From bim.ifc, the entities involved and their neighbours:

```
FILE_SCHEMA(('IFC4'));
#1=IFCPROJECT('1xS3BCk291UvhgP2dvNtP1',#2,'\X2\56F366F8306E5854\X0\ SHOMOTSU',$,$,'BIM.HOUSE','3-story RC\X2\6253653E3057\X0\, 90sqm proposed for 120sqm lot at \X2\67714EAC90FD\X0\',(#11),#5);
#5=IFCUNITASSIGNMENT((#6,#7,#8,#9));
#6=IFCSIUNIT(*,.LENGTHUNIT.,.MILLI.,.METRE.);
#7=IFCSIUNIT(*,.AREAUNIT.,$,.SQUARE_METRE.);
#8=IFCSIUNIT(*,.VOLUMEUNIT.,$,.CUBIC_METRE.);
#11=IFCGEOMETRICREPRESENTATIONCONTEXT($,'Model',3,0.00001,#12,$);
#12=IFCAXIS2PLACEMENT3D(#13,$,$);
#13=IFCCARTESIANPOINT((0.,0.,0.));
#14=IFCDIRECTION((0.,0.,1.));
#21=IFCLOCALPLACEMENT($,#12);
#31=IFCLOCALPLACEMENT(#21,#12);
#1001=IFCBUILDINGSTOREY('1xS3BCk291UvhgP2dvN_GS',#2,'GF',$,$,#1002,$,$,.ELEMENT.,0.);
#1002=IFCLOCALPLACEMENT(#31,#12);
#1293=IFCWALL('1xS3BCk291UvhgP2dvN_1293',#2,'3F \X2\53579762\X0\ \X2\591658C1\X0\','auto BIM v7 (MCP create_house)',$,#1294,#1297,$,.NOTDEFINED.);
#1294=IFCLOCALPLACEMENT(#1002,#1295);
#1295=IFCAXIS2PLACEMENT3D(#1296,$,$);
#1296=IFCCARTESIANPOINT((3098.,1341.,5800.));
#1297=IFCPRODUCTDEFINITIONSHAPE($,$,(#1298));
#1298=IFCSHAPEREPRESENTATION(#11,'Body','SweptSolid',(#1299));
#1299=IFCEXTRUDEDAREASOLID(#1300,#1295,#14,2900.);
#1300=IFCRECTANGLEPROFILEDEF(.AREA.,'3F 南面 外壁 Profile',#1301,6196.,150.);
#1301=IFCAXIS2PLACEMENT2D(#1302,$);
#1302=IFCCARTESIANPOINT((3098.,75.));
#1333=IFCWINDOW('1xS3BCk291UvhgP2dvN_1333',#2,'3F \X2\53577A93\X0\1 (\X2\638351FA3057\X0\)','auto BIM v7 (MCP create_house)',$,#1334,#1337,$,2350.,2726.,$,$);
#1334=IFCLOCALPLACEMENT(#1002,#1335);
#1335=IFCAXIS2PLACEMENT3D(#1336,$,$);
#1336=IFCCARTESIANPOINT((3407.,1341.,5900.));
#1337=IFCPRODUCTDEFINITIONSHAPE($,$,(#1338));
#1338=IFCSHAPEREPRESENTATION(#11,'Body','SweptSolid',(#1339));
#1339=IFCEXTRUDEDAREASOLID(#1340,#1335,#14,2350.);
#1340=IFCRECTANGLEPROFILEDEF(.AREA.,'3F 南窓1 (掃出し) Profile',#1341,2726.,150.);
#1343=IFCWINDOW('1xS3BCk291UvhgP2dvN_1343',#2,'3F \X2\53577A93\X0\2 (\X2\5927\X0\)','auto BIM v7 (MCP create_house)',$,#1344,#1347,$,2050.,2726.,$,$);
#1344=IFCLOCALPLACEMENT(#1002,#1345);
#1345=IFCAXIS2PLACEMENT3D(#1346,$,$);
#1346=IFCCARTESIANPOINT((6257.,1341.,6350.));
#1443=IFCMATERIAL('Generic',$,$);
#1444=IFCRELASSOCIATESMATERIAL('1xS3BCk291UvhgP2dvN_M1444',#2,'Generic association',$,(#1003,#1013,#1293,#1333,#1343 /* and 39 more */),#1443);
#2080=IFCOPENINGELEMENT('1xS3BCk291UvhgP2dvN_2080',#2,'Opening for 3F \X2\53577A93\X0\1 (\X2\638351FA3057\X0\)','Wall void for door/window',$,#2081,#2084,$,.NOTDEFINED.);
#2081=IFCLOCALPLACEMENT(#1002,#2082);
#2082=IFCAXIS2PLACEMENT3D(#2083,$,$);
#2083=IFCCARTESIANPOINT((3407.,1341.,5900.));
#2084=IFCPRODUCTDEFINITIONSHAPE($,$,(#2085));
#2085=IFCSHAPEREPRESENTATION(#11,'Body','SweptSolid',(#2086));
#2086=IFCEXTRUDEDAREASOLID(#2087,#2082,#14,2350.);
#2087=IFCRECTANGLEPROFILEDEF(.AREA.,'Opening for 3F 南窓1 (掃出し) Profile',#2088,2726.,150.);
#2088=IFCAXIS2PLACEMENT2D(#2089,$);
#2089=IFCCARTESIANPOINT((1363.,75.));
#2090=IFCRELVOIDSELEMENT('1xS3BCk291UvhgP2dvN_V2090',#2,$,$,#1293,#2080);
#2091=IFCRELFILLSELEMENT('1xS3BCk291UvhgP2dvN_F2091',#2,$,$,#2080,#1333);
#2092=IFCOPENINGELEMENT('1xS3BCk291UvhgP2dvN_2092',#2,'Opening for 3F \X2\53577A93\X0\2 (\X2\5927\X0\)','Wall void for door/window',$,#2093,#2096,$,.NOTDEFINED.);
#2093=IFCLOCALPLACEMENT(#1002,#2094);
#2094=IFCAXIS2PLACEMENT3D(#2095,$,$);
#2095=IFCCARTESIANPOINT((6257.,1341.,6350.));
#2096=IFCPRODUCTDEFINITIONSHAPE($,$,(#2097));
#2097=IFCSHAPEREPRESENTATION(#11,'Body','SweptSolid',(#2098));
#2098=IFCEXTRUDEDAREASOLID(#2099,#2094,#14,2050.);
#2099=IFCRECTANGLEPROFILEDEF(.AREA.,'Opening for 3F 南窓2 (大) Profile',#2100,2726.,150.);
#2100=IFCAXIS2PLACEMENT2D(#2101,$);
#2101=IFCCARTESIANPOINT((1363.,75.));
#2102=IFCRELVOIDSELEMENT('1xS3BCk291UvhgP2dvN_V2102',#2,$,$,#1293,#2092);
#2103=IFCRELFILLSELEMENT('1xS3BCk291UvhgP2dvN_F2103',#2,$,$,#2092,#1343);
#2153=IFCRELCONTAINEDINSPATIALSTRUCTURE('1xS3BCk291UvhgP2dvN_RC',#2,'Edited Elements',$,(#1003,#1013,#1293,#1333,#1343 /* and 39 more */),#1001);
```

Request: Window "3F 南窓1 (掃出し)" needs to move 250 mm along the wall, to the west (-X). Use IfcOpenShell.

```python
import ifcopenshell
import ifcopenshell.api.geometry
import ifcopenshell.util.placement

model = ifcopenshell.open("bim.ifc")

window = model.by_guid("1xS3BCk291UvhgP2dvN_1333")
opening = window.FillsVoids[0].RelatingOpeningElement
wall = opening.VoidsElements[0].RelatingBuildingElement

wall_matrix = ifcopenshell.util.placement.get_local_placement(wall.ObjectPlacement)
shift = wall_matrix[:3, 0] * -250.0
before = ifcopenshell.util.placement.get_local_placement(window.ObjectPlacement)[:3, 3].copy()

# The window is not placed relative to its opening, so move both.
for product in (opening, window):
    matrix = ifcopenshell.util.placement.get_local_placement(product.ObjectPlacement)
    matrix[:3, 3] += shift
    ifcopenshell.api.geometry.edit_object_placement(model, product=product, matrix=matrix, is_si=False)

after = ifcopenshell.util.placement.get_local_placement(window.ObjectPlacement)[:3, 3]
print("window moved by", (after - before).round(3) + 0.0)

model.write("bim-out.ifc")
```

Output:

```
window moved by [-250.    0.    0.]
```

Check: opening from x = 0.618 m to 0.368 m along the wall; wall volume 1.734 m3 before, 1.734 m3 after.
